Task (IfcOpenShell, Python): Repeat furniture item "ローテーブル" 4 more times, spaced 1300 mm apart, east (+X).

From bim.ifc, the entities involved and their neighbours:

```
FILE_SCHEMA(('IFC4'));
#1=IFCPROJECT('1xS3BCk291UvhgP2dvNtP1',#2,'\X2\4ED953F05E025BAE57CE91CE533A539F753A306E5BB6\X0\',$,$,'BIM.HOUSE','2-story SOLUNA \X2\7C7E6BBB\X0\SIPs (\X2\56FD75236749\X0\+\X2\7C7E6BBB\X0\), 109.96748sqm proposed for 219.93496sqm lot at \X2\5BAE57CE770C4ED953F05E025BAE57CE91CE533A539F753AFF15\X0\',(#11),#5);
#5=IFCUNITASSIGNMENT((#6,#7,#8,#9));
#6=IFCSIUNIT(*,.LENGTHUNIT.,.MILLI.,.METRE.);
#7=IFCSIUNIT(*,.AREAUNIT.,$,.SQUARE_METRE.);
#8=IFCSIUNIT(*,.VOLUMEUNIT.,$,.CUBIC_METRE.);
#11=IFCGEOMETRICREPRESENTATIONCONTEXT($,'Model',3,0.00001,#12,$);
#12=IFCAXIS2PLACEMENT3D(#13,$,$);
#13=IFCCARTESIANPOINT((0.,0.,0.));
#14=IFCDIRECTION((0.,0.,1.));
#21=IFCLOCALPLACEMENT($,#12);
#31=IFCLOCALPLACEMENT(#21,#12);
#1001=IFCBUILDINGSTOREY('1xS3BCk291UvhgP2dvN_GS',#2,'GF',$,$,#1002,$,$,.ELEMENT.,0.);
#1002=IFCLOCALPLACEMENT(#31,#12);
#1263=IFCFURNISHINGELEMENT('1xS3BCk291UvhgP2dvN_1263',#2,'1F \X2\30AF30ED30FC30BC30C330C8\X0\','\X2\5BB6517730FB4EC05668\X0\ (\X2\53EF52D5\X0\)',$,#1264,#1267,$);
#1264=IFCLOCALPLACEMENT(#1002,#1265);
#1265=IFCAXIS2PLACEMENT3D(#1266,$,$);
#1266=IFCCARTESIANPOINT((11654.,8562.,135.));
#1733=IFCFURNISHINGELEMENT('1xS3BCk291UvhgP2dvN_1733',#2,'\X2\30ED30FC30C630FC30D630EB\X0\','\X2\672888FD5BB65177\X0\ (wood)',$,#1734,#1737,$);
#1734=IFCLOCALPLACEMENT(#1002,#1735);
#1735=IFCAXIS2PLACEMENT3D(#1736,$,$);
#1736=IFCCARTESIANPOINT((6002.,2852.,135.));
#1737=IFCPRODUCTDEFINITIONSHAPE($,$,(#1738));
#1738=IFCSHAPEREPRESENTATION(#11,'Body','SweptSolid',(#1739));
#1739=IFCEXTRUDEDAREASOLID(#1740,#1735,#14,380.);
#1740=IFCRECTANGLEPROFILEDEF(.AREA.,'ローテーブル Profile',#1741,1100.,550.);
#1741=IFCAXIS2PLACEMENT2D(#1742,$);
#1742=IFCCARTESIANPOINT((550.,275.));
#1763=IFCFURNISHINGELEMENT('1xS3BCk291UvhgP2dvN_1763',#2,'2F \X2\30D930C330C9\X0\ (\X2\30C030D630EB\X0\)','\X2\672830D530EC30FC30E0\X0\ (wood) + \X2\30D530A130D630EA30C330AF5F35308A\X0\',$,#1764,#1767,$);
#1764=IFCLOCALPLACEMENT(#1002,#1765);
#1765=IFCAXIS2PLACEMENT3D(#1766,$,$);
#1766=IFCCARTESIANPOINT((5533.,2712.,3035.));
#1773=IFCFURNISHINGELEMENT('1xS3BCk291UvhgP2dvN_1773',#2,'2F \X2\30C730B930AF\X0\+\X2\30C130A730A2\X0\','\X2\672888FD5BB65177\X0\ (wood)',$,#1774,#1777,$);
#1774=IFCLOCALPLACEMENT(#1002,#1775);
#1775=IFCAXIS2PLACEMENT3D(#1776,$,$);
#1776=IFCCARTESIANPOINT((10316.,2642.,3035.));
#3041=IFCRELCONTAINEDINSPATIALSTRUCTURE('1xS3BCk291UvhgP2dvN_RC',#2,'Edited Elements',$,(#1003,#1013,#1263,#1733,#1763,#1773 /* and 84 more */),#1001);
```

```python
import numpy as np
import ifcopenshell
import ifcopenshell.api.geometry
import ifcopenshell.api.root
import ifcopenshell.util.element
import ifcopenshell.util.placement
import ifcopenshell.util.unit

model = ifcopenshell.open("bim.ifc")
unit_scale = ifcopenshell.util.unit.calculate_unit_scale(model)


def reuse_history(source, copy):
    """copy_class also copies each property set's owner history, people and application; keep the originals."""
    for rel in copy.IsDefinedBy:
        if rel.is_a("IfcRelDefinesByProperties") and (history := rel.RelatingPropertyDefinition.OwnerHistory):
            rel.RelatingPropertyDefinition.OwnerHistory = source.OwnerHistory
            ifcopenshell.util.element.remove_deep2(model, history)


source = model.by_guid("1xS3BCk291UvhgP2dvN_1733")
base = ifcopenshell.util.placement.get_local_placement(source.ObjectPlacement)
step = np.array([1.0, 0.0, 0.0]) * 1.3 / unit_scale

for i in range(1, 5):
    copy = ifcopenshell.api.root.copy_class(model, product=source)
    copy.Representation = ifcopenshell.util.element.copy_deep(
        model, source.Representation, exclude=["IfcGeometricRepresentationContext", "IfcRepresentationMap"]
    )
    reuse_history(source, copy)
    matrix = base.copy()
    matrix[:3, 3] += i * step
    print("added at", matrix[:3, 3].round(3) + 0.0)
    ifcopenshell.api.geometry.edit_object_placement(model, product=copy, matrix=matrix, is_si=False)

model.write("bim_v2.ifc")
```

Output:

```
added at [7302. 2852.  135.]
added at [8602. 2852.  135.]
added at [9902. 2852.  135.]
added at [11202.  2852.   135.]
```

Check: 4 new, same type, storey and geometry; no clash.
